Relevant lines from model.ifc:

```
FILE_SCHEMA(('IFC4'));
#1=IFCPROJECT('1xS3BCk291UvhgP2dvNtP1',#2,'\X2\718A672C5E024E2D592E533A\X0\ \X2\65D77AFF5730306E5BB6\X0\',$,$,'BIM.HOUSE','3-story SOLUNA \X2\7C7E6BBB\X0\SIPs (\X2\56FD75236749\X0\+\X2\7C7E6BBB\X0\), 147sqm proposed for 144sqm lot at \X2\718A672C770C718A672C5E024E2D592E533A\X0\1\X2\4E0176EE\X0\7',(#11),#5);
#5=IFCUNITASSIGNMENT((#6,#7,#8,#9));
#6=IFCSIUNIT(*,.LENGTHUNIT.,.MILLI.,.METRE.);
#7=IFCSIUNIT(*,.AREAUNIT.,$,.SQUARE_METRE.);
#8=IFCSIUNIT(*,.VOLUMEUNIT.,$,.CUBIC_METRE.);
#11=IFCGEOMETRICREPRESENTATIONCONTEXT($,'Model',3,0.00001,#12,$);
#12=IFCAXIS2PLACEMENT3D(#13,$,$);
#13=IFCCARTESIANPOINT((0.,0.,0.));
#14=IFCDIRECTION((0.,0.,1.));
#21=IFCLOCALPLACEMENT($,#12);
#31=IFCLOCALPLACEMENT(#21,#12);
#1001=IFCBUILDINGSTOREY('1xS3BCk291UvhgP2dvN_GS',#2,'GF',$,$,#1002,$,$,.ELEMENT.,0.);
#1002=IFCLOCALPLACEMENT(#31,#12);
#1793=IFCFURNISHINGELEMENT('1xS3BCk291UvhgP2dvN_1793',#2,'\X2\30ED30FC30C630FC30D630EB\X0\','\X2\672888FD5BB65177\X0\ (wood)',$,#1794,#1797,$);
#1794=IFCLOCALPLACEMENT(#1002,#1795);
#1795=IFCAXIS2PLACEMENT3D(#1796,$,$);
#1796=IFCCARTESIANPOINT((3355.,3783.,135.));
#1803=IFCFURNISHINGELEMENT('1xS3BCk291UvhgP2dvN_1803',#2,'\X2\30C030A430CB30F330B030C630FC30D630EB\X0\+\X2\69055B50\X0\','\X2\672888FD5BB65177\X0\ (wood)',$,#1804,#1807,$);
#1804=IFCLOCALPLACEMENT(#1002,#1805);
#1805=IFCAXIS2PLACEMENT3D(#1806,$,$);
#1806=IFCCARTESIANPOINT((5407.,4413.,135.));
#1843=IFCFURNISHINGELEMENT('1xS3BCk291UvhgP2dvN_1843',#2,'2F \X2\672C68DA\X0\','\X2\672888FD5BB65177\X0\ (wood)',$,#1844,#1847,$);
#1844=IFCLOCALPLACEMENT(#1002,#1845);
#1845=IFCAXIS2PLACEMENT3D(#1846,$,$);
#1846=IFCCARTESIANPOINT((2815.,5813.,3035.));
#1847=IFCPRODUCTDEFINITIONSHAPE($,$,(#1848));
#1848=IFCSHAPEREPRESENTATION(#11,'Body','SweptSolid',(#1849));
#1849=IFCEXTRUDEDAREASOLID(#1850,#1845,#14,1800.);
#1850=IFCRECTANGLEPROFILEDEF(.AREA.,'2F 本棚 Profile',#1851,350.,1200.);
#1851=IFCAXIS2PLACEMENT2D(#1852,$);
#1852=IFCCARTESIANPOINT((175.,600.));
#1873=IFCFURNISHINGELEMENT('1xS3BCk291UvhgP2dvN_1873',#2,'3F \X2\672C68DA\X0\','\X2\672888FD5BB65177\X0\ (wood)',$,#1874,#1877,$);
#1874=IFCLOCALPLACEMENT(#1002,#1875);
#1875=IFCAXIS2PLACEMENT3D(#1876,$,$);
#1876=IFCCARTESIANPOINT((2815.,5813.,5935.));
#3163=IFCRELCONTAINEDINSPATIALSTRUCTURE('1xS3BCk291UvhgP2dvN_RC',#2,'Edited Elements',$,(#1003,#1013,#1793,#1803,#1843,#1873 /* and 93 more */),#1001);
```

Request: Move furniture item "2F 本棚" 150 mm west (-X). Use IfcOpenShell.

```python
import ifcopenshell
import ifcopenshell.api.geometry
import ifcopenshell.util.placement

model = ifcopenshell.open("model.ifc")

item = model.by_guid("1xS3BCk291UvhgP2dvN_1843")
matrix = ifcopenshell.util.placement.get_local_placement(item.ObjectPlacement)
matrix[0, 3] -= 150.0
ifcopenshell.api.geometry.edit_object_placement(model, product=item, matrix=matrix, is_si=False)

print(ifcopenshell.util.placement.get_local_placement(item.ObjectPlacement).round(3) + 0.0)

model.write("model_edited.ifc")
```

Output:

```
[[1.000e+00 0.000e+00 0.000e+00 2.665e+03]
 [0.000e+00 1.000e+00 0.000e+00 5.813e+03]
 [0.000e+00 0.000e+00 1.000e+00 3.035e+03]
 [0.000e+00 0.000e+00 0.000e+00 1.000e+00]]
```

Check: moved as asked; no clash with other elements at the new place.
